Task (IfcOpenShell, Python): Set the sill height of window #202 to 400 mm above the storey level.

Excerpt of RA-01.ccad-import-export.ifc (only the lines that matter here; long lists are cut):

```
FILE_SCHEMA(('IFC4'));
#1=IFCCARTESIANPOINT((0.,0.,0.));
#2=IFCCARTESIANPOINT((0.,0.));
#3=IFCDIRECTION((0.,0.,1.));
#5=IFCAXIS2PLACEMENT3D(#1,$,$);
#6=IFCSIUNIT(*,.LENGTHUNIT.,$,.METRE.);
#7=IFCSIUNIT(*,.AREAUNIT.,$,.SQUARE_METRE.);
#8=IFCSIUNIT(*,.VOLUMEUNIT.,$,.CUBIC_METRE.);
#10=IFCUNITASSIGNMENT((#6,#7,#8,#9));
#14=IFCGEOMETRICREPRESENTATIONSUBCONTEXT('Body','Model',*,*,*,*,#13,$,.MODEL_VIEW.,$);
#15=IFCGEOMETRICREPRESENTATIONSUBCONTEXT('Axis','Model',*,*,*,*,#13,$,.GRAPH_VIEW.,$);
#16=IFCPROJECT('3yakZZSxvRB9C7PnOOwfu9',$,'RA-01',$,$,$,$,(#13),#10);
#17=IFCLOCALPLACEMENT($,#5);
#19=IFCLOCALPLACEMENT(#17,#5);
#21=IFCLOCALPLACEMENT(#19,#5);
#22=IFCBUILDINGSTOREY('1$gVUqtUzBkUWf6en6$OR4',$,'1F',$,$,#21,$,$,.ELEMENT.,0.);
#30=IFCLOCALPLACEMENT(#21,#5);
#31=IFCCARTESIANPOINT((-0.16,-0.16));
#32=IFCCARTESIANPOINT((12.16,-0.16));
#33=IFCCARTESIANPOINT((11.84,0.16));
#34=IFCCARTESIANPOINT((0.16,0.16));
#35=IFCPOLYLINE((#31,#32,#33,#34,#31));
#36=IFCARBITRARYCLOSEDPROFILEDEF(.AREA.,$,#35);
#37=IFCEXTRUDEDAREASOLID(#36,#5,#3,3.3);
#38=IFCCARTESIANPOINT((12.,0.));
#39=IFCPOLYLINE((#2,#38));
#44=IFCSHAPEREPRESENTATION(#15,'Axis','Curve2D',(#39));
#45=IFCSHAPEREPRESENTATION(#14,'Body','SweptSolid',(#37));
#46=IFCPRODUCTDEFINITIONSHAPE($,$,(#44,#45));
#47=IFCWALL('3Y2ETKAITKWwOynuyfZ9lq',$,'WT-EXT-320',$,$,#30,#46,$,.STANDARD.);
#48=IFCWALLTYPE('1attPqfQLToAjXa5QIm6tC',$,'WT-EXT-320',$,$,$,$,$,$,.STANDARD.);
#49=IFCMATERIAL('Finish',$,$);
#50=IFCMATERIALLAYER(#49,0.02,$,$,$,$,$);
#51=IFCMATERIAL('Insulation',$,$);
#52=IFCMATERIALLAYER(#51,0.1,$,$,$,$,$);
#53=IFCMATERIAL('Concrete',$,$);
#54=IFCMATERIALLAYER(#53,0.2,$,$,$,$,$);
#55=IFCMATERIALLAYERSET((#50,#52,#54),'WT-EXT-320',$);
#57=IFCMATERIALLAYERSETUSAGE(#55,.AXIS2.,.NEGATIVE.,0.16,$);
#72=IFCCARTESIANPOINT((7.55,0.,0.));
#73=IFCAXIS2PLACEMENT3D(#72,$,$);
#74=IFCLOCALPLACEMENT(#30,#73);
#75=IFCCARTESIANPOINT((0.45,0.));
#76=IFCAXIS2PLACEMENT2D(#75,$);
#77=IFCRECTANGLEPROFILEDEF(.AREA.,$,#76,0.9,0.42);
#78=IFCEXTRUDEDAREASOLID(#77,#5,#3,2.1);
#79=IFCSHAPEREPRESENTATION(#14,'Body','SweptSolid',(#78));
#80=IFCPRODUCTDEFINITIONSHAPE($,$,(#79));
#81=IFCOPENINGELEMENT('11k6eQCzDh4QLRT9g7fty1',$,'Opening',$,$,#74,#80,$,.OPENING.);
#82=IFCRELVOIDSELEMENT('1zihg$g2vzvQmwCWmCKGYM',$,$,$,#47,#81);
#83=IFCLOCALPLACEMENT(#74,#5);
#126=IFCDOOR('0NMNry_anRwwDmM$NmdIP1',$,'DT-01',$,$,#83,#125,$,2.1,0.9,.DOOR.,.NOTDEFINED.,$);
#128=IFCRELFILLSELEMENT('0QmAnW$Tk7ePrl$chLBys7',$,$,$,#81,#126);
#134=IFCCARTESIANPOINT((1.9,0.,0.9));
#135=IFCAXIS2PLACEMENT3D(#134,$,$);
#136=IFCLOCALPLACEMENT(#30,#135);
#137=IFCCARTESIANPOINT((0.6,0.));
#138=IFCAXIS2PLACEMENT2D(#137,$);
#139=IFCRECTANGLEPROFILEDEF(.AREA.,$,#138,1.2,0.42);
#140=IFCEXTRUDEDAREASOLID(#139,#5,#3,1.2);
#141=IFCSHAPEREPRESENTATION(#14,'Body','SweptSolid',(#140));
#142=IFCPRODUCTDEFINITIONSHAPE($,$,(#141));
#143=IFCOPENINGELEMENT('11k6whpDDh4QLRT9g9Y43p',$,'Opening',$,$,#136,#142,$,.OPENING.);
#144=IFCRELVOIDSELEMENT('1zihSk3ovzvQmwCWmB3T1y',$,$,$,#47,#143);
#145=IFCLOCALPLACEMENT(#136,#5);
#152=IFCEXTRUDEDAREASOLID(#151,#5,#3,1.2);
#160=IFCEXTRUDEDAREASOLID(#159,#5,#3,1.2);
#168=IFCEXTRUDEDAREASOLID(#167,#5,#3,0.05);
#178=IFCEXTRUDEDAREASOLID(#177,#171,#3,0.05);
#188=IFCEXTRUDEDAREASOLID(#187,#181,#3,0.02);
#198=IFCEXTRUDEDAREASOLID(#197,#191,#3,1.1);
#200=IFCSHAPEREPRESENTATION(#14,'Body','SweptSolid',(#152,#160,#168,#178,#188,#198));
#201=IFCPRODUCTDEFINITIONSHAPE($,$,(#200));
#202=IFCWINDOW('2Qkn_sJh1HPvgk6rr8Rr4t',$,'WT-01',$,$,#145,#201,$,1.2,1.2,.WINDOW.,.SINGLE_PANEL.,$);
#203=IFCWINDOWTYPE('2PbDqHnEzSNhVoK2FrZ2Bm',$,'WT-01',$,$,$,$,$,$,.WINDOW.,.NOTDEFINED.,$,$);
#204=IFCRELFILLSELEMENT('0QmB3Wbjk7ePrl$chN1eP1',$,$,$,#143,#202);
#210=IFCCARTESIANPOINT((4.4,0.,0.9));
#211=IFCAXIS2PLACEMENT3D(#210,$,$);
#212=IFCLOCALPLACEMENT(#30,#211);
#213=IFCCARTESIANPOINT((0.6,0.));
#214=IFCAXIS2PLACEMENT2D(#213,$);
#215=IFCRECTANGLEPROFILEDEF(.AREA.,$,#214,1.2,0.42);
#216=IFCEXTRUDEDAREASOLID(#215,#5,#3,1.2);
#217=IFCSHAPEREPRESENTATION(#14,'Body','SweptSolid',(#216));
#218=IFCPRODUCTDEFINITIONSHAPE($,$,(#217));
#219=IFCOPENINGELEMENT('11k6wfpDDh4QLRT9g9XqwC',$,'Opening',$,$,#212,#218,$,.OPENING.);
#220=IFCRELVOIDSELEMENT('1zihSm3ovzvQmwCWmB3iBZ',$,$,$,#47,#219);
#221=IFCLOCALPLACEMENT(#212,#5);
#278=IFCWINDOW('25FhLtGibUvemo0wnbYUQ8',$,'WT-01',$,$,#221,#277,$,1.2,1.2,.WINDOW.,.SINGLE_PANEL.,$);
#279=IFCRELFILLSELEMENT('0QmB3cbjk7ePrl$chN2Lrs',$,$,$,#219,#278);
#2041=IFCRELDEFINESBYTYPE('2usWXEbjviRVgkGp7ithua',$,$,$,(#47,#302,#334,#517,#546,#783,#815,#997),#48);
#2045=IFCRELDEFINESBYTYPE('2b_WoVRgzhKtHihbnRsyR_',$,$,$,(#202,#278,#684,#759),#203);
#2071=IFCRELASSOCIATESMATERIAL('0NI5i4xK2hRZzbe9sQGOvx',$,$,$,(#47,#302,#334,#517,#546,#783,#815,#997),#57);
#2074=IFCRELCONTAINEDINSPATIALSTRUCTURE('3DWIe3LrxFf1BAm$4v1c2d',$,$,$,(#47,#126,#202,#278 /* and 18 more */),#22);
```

```python
import numpy as np
import ifcopenshell
import ifcopenshell.api.geometry
import ifcopenshell.geom
import ifcopenshell.util.element
import ifcopenshell.util.placement
import ifcopenshell.util.shape
import ifcopenshell.util.unit

model = ifcopenshell.open("RA-01.ccad-import-export.ifc")
unit_scale = ifcopenshell.util.unit.calculate_unit_scale(model)

window = model.by_id(202)
opening = window.FillsVoids[0].RelatingOpeningElement
storey = ifcopenshell.util.element.get_container(window, ifc_class="IfcBuildingStorey")
level = ifcopenshell.util.placement.get_local_placement(storey.ObjectPlacement)[2, 3]

# The opening's origin need not be at the sill, so measure its lowest point.
shape = ifcopenshell.geom.create_shape(ifcopenshell.geom.settings(), opening)
bottom = ifcopenshell.util.shape.get_shape_bottom_elevation(shape, shape.geometry) / unit_scale
dz = level + 0.4 - bottom

shift = np.array([0.0, 0.0, dz])
# The window is placed relative to its opening, so it follows when the opening moves.
matrix = ifcopenshell.util.placement.get_local_placement(opening.ObjectPlacement)
matrix[:3, 3] += shift
ifcopenshell.api.geometry.edit_object_placement(
    model, product=opening, matrix=matrix, is_si=False, should_transform_children=True
)

print(f"moved by {dz * unit_scale:+.3f} m")

model.write("RA-01.ccad-import-export_rev.ifc")
```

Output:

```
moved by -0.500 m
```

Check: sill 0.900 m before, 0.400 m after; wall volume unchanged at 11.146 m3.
